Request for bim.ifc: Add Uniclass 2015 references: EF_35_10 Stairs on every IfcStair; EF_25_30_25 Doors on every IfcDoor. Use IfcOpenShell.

First a look at what the model holds.

```python
import ifcopenshell

model = ifcopenshell.open("bim.ifc")
print(model.schema)
print("classifications:", [c.Name for c in model.by_type("IfcClassification")])
for ifc_class in ("IfcDoor", "IfcRoof", "IfcStair", "IfcWall", "IfcWindow"):
    print(ifc_class, len(model.by_type(ifc_class)))
```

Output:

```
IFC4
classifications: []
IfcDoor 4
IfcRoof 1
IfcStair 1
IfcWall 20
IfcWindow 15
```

```python
import ifcopenshell
import ifcopenshell.api.classification

model = ifcopenshell.open("bim.ifc")

system = ifcopenshell.api.classification.add_classification(model, classification="Uniclass 2015")

codes = {
    "IfcStair": ("EF_35_10", "Stairs"),
    "IfcDoor": ("EF_25_30_25", "Doors"),
}
for ifc_class, (code, name) in codes.items():
    products = model.by_type(ifc_class)
    ifcopenshell.api.classification.add_reference(
        model, products=products, classification=system, identification=code, name=name
    )
    print(code, len(products))

model.write("bim_rev.ifc")
```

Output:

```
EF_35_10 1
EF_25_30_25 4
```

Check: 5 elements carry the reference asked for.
